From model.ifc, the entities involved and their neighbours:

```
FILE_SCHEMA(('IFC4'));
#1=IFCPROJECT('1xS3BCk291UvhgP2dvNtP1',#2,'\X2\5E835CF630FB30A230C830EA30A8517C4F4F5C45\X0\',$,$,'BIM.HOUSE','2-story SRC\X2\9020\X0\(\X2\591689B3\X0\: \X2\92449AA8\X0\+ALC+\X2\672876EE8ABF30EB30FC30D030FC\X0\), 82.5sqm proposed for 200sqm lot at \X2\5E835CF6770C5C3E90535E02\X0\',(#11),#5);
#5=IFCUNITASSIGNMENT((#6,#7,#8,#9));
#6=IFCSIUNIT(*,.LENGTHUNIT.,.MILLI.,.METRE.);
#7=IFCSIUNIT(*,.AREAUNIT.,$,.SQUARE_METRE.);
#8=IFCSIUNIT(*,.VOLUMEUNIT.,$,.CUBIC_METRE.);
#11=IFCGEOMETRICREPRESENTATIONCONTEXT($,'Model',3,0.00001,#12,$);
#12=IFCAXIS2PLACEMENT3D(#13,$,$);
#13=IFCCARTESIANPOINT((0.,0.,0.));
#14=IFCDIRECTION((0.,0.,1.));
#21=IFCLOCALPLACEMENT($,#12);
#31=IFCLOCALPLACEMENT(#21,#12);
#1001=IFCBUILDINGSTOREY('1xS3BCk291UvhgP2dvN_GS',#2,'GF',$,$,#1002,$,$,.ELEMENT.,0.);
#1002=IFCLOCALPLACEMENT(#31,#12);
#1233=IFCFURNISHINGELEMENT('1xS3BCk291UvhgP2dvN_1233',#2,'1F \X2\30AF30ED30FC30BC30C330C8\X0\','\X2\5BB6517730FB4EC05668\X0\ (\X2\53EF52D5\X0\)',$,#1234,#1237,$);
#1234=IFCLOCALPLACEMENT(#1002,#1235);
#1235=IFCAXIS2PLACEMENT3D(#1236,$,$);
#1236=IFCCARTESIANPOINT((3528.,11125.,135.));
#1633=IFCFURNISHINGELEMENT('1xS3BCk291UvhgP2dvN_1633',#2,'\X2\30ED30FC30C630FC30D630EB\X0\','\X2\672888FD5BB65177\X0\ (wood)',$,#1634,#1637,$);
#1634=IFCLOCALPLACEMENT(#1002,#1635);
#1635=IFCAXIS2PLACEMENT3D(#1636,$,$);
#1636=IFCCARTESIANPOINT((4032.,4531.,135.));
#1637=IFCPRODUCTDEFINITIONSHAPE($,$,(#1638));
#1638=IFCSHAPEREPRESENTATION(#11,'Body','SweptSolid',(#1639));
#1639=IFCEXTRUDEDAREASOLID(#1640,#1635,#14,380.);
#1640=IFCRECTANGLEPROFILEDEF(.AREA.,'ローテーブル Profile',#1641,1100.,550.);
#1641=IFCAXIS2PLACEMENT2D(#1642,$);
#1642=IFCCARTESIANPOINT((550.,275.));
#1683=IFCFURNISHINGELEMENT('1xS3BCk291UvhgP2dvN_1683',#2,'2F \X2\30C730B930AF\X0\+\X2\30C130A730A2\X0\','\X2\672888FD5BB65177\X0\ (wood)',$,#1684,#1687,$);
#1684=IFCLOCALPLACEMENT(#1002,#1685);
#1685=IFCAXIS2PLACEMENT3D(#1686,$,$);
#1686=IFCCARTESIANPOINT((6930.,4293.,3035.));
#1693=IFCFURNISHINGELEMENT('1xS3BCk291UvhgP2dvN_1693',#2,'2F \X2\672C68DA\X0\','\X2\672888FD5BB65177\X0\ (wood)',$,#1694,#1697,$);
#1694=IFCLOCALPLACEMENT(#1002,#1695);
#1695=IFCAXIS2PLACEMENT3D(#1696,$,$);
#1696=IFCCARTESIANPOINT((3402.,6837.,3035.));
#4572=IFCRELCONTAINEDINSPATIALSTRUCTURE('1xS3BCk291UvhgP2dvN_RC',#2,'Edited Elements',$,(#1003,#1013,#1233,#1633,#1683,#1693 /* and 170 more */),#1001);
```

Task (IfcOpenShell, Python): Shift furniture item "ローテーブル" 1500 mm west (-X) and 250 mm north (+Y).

```python
import ifcopenshell
import ifcopenshell.api.geometry
import ifcopenshell.util.placement
import ifcopenshell.util.unit

model = ifcopenshell.open("model.ifc")
unit_scale = ifcopenshell.util.unit.calculate_unit_scale(model)

item = model.by_guid("1xS3BCk291UvhgP2dvN_1633")
matrix = ifcopenshell.util.placement.get_local_placement(item.ObjectPlacement)
matrix[0, 3] -= 1.5 / unit_scale
matrix[1, 3] += 0.25 / unit_scale
ifcopenshell.api.geometry.edit_object_placement(model, product=item, matrix=matrix, is_si=False)

print(ifcopenshell.util.placement.get_local_placement(item.ObjectPlacement).round(3) + 0.0)

model.write("model_updated.ifc")
```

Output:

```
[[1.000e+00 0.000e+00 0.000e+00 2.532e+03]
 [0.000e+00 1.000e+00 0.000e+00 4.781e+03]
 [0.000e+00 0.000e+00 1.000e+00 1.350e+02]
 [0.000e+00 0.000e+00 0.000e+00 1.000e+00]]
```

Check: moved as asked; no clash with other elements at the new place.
